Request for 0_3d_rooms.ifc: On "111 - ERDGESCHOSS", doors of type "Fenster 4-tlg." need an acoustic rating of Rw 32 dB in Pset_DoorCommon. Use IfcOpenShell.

First a look at what the model holds.

```python
import ifcopenshell
import ifcopenshell.util.element

model = ifcopenshell.open("0_3d_rooms.ifc")
print(model.schema)
storey = next(s for s in model.by_type("IfcBuildingStorey") if s.Name == "111 - ERDGESCHOSS")
doors = [e for e in ifcopenshell.util.element.get_decomposition(storey) if e.is_a("IfcDoor")]
seen = {}
for e in doors:
    element_type = ifcopenshell.util.element.get_type(e)
    key = (element_type.Name if element_type != e and element_type else None, ifcopenshell.util.element.get_pset(e, "Pset_DoorCommon", "AcousticRating"))
    seen[key] = seen.get(key, 0) + 1
for (name, value), count in sorted(seen.items(), key=str):
    print(count, "x", name, "|", value)
```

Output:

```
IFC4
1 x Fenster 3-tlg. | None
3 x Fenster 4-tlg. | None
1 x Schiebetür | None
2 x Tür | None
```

```python
import ifcopenshell
import ifcopenshell.api.pset
import ifcopenshell.util.element

model = ifcopenshell.open("0_3d_rooms.ifc")

storey = next(s for s in model.by_type("IfcBuildingStorey") if s.Name == "111 - ERDGESCHOSS")
doors = [e for e in ifcopenshell.util.element.get_decomposition(storey) if e.is_a("IfcDoor")]

count = 0
for e in doors:
    element_type = ifcopenshell.util.element.get_type(e)
    if element_type in (None, e) or element_type.Name != "Fenster 4-tlg.":
        continue
    # add_pset returns the element's existing set when there is one.
    pset = ifcopenshell.api.pset.add_pset(model, product=e, name="Pset_DoorCommon")
    ifcopenshell.api.pset.edit_pset(model, pset=pset, properties={"AcousticRating": "Rw 32 dB"})
    count += 1

print(count, "doors updated")

model.write("0_3d_rooms_updated.ifc")
```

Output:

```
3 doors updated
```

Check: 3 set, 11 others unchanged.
